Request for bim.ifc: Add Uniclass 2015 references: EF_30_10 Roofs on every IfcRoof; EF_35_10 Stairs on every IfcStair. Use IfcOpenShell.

First a look at what the model holds.

```python
import ifcopenshell

model = ifcopenshell.open("bim.ifc")
print(model.schema)
print("classifications:", [c.Name for c in model.by_type("IfcClassification")])
for ifc_class in ("IfcDoor", "IfcRoof", "IfcStair", "IfcWall", "IfcWindow"):
    print(ifc_class, len(model.by_type(ifc_class)))
```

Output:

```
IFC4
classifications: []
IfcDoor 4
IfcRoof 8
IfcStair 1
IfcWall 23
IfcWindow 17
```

```python
import ifcopenshell
import ifcopenshell.api.classification

model = ifcopenshell.open("bim.ifc")

system = ifcopenshell.api.classification.add_classification(model, classification="Uniclass 2015")

codes = {
    "IfcRoof": ("EF_30_10", "Roofs"),
    "IfcStair": ("EF_35_10", "Stairs"),
}
for ifc_class, (code, name) in codes.items():
    products = model.by_type(ifc_class)
    ifcopenshell.api.classification.add_reference(
        model, products=products, classification=system, identification=code, name=name
    )
    print(code, len(products))

model.write("bim-out.ifc")
```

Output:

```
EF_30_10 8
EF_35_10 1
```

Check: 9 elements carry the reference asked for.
